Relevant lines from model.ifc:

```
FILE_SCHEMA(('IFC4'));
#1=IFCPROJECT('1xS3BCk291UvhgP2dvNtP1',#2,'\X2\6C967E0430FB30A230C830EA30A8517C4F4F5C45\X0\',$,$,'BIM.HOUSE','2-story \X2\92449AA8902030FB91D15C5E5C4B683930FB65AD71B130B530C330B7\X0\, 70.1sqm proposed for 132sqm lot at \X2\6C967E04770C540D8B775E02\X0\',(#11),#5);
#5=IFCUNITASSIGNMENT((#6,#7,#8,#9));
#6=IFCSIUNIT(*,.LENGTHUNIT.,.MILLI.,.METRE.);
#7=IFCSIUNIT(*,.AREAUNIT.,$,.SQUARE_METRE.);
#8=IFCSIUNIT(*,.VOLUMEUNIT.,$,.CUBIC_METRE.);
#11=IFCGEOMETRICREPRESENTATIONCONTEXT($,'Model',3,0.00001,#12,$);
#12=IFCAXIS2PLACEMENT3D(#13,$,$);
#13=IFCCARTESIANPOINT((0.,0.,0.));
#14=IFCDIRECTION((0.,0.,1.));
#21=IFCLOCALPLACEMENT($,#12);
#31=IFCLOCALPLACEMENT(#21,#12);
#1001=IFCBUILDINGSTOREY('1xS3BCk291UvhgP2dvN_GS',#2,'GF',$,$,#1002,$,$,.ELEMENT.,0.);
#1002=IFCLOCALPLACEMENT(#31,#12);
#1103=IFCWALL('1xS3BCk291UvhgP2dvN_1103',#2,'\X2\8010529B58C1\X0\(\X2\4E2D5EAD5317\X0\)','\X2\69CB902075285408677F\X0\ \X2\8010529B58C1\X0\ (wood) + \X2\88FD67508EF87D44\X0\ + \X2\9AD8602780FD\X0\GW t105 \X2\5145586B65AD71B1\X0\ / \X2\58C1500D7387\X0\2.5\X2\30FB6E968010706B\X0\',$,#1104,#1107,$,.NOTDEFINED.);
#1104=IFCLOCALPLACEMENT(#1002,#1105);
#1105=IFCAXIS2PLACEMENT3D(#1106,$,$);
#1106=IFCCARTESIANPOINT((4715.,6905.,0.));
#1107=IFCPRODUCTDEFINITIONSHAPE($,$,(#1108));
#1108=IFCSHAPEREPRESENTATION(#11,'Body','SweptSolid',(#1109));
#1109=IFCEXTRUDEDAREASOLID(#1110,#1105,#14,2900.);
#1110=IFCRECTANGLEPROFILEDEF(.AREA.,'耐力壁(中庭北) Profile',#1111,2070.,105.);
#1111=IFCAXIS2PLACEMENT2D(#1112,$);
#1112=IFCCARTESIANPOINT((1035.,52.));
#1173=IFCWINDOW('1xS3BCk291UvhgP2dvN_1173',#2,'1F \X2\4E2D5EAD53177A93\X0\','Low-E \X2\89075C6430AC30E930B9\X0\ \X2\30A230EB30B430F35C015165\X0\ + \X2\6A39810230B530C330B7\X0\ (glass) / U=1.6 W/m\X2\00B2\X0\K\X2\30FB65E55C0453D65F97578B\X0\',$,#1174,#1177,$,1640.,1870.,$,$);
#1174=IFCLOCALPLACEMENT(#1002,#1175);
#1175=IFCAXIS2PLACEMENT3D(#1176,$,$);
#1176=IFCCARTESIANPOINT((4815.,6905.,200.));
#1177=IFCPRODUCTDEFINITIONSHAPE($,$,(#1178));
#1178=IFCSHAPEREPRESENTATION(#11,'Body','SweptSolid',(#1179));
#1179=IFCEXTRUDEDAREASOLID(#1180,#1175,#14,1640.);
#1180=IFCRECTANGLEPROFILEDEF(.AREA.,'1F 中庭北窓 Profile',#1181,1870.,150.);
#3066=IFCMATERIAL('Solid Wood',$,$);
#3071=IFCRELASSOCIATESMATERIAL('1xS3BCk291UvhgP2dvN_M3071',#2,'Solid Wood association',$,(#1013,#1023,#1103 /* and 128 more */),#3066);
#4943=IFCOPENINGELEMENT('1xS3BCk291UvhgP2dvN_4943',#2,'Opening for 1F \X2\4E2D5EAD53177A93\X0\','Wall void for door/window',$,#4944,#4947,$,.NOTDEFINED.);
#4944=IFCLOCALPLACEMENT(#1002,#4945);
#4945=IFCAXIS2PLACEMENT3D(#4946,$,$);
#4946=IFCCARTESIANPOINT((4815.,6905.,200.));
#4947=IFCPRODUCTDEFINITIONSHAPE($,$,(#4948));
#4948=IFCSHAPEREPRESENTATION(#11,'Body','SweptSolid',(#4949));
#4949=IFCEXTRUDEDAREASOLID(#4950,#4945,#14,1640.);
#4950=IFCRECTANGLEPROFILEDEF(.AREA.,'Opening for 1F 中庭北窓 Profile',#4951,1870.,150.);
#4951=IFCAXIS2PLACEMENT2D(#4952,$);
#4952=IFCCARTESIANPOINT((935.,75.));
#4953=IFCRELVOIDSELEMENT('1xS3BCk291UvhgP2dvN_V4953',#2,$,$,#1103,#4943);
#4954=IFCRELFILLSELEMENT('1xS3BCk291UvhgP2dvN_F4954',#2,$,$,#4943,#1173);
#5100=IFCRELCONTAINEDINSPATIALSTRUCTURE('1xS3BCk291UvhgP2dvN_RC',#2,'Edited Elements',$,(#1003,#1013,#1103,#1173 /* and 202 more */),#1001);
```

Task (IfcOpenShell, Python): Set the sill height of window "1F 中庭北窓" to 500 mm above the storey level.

```python
import numpy as np
import ifcopenshell
import ifcopenshell.api.geometry
import ifcopenshell.geom
import ifcopenshell.util.element
import ifcopenshell.util.placement
import ifcopenshell.util.shape
import ifcopenshell.util.unit

model = ifcopenshell.open("model.ifc")
unit_scale = ifcopenshell.util.unit.calculate_unit_scale(model)

window = model.by_id(1173)
opening = window.FillsVoids[0].RelatingOpeningElement
storey = ifcopenshell.util.element.get_container(window, ifc_class="IfcBuildingStorey")
level = ifcopenshell.util.placement.get_local_placement(storey.ObjectPlacement)[2, 3]

# The opening's origin need not be at the sill, so measure its lowest point.
shape = ifcopenshell.geom.create_shape(ifcopenshell.geom.settings(), opening)
bottom = ifcopenshell.util.shape.get_shape_bottom_elevation(shape, shape.geometry) / unit_scale
dz = level + 0.5 / unit_scale - bottom

shift = np.array([0.0, 0.0, dz])
# The window is not placed relative to its opening, so move both.
for product in (opening, window):
    matrix = ifcopenshell.util.placement.get_local_placement(product.ObjectPlacement)
    matrix[:3, 3] += shift
    ifcopenshell.api.geometry.edit_object_placement(model, product=product, matrix=matrix, is_si=False)

print(f"moved by {dz * unit_scale:+.3f} m")

model.write("model-out.ifc")
```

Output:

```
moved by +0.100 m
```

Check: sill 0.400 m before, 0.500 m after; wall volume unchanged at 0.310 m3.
